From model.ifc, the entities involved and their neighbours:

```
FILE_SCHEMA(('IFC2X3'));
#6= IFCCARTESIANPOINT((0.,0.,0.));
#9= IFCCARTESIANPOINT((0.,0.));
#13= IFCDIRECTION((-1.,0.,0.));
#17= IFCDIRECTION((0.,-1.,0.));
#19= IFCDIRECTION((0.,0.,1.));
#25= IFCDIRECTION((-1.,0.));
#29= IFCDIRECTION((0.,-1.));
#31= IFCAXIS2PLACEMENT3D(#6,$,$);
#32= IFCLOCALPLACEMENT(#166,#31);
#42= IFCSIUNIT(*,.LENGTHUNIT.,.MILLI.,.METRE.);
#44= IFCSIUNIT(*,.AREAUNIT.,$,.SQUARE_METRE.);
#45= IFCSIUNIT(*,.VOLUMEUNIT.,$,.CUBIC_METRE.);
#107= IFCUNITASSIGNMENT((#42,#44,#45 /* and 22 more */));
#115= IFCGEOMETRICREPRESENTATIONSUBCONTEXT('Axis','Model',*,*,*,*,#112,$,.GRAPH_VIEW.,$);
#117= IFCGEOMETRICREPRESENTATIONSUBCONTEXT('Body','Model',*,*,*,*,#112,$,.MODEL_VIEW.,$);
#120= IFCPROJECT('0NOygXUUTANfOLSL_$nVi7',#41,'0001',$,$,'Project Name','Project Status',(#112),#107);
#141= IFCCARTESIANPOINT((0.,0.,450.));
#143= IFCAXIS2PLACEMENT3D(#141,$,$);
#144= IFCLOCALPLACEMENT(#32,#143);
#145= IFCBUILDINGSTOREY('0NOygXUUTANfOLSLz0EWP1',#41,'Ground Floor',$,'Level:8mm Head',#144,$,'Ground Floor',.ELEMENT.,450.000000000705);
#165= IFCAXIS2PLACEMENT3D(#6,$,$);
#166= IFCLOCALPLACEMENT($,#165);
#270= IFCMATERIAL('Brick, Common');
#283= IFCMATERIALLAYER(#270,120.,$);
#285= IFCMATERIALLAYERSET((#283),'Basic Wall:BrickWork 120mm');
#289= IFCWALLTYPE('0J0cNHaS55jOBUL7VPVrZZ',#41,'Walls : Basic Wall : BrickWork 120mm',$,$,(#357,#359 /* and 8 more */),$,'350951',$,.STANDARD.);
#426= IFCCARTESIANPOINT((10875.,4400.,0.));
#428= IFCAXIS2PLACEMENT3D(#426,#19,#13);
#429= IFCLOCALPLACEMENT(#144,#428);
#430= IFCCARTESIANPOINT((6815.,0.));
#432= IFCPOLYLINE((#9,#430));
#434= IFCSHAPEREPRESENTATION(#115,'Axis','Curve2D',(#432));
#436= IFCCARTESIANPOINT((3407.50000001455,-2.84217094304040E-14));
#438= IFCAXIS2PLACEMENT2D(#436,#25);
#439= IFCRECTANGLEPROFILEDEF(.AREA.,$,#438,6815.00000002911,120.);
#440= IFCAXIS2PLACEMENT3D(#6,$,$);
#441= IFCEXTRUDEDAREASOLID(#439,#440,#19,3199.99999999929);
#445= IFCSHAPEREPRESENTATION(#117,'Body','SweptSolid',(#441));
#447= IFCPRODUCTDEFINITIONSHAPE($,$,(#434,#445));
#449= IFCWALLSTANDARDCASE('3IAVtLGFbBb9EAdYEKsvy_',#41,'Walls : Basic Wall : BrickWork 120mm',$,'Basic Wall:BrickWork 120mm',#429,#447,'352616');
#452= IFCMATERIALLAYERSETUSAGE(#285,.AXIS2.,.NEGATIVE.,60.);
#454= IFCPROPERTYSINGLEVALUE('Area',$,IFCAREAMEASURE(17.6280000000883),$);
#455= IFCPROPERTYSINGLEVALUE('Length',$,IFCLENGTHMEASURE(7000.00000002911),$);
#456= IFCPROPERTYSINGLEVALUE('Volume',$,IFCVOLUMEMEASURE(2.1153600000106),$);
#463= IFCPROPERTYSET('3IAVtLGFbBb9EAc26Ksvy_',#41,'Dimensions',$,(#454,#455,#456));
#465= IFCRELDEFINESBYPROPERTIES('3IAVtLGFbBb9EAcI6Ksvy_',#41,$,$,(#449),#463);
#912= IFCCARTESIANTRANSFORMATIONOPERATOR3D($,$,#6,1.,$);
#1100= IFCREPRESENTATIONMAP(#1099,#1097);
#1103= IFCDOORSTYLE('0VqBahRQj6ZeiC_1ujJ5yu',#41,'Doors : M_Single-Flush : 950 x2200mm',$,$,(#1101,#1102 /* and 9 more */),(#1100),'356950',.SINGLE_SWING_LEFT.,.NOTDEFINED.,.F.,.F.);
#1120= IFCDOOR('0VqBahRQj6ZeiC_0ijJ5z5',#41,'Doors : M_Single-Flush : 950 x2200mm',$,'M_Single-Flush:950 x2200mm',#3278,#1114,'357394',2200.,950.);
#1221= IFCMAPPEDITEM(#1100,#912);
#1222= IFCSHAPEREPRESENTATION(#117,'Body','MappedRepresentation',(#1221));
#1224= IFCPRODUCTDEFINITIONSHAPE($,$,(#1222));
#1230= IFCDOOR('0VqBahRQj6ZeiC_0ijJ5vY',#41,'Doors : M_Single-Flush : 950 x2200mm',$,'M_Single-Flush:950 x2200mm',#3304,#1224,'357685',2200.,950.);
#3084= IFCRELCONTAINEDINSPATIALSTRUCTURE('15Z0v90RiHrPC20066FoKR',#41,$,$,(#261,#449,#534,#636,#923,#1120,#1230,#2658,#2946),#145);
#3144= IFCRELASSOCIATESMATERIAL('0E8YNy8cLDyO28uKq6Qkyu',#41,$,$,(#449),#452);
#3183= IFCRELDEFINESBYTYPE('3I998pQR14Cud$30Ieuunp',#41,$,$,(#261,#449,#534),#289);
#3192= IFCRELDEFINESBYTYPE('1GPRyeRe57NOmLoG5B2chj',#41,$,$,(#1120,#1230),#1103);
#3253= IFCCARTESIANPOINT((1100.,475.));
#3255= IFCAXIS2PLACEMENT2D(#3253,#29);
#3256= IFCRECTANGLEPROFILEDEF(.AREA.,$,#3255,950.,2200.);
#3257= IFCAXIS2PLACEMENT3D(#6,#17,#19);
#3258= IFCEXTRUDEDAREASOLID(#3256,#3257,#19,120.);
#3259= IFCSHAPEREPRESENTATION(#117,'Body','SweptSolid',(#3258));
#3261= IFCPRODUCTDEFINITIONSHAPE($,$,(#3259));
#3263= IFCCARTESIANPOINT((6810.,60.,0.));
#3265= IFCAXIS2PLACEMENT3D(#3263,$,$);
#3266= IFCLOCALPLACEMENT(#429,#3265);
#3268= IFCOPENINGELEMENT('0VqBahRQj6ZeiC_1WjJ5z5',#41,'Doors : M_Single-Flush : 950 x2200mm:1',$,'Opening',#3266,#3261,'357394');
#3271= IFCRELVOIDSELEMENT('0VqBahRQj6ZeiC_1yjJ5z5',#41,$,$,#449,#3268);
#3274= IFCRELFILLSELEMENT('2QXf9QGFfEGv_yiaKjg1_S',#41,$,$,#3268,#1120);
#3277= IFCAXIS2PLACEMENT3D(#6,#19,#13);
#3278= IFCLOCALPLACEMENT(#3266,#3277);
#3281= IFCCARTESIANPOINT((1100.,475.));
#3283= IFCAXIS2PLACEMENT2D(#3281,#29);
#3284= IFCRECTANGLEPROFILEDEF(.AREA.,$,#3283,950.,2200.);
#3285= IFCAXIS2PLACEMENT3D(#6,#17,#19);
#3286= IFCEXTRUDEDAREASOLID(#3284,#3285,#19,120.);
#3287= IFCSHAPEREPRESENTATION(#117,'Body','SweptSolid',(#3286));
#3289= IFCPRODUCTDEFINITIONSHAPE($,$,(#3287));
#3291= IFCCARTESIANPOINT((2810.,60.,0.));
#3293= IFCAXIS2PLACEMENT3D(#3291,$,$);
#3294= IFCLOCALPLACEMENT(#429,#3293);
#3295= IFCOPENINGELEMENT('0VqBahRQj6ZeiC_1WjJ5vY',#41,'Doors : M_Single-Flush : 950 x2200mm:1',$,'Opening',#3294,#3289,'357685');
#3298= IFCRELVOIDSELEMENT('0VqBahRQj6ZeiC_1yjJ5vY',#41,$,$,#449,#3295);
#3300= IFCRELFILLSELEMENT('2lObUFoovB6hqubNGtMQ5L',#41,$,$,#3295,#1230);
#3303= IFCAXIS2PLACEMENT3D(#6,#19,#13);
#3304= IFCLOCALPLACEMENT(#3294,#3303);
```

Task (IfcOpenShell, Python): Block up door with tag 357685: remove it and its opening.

```python
import ifcopenshell
import ifcopenshell.api.feature
import ifcopenshell.api.pset
import ifcopenshell.api.root
import ifcopenshell.geom
import ifcopenshell.util.element
import ifcopenshell.util.shape
import ifcopenshell.util.unit

model = ifcopenshell.open("model.ifc")
area_scale = ifcopenshell.util.unit.calculate_unit_scale(model, "AREAUNIT")
volume_scale = ifcopenshell.util.unit.calculate_unit_scale(model, "VOLUMEUNIT")
settings = ifcopenshell.geom.settings()


def volume(element):
    """Net volume in cubic metres, openings subtracted."""
    shape = ifcopenshell.geom.create_shape(settings, element)
    return ifcopenshell.util.shape.get_volume(shape.geometry)


door = model.by_id(1230)
opening = door.FillsVoids[0].RelatingOpeningElement
wall = opening.VoidsElements[0].RelatingBuildingElement
before = volume(wall)

ifcopenshell.api.root.remove_product(model, product=door)
ifcopenshell.api.feature.remove_feature(model, feature=opening)

after = volume(wall)
thickness = 0.12  # wall thickness in metres

# Update the wall's stored quantities.
pset = model.by_id(ifcopenshell.util.element.get_pset(wall, "Dimensions", should_inherit=False)["id"])
ifcopenshell.api.pset.edit_pset(model, pset=pset, properties={
    "Area": model.create_entity("IfcAreaMeasure", after / thickness / area_scale),
    "Volume": model.create_entity("IfcVolumeMeasure", after / volume_scale),
})

print(f"wall volume {before:.3f} -> {after:.3f} m3")

model.write("model-out.ifc")
```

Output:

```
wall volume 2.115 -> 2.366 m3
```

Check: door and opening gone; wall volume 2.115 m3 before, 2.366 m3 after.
